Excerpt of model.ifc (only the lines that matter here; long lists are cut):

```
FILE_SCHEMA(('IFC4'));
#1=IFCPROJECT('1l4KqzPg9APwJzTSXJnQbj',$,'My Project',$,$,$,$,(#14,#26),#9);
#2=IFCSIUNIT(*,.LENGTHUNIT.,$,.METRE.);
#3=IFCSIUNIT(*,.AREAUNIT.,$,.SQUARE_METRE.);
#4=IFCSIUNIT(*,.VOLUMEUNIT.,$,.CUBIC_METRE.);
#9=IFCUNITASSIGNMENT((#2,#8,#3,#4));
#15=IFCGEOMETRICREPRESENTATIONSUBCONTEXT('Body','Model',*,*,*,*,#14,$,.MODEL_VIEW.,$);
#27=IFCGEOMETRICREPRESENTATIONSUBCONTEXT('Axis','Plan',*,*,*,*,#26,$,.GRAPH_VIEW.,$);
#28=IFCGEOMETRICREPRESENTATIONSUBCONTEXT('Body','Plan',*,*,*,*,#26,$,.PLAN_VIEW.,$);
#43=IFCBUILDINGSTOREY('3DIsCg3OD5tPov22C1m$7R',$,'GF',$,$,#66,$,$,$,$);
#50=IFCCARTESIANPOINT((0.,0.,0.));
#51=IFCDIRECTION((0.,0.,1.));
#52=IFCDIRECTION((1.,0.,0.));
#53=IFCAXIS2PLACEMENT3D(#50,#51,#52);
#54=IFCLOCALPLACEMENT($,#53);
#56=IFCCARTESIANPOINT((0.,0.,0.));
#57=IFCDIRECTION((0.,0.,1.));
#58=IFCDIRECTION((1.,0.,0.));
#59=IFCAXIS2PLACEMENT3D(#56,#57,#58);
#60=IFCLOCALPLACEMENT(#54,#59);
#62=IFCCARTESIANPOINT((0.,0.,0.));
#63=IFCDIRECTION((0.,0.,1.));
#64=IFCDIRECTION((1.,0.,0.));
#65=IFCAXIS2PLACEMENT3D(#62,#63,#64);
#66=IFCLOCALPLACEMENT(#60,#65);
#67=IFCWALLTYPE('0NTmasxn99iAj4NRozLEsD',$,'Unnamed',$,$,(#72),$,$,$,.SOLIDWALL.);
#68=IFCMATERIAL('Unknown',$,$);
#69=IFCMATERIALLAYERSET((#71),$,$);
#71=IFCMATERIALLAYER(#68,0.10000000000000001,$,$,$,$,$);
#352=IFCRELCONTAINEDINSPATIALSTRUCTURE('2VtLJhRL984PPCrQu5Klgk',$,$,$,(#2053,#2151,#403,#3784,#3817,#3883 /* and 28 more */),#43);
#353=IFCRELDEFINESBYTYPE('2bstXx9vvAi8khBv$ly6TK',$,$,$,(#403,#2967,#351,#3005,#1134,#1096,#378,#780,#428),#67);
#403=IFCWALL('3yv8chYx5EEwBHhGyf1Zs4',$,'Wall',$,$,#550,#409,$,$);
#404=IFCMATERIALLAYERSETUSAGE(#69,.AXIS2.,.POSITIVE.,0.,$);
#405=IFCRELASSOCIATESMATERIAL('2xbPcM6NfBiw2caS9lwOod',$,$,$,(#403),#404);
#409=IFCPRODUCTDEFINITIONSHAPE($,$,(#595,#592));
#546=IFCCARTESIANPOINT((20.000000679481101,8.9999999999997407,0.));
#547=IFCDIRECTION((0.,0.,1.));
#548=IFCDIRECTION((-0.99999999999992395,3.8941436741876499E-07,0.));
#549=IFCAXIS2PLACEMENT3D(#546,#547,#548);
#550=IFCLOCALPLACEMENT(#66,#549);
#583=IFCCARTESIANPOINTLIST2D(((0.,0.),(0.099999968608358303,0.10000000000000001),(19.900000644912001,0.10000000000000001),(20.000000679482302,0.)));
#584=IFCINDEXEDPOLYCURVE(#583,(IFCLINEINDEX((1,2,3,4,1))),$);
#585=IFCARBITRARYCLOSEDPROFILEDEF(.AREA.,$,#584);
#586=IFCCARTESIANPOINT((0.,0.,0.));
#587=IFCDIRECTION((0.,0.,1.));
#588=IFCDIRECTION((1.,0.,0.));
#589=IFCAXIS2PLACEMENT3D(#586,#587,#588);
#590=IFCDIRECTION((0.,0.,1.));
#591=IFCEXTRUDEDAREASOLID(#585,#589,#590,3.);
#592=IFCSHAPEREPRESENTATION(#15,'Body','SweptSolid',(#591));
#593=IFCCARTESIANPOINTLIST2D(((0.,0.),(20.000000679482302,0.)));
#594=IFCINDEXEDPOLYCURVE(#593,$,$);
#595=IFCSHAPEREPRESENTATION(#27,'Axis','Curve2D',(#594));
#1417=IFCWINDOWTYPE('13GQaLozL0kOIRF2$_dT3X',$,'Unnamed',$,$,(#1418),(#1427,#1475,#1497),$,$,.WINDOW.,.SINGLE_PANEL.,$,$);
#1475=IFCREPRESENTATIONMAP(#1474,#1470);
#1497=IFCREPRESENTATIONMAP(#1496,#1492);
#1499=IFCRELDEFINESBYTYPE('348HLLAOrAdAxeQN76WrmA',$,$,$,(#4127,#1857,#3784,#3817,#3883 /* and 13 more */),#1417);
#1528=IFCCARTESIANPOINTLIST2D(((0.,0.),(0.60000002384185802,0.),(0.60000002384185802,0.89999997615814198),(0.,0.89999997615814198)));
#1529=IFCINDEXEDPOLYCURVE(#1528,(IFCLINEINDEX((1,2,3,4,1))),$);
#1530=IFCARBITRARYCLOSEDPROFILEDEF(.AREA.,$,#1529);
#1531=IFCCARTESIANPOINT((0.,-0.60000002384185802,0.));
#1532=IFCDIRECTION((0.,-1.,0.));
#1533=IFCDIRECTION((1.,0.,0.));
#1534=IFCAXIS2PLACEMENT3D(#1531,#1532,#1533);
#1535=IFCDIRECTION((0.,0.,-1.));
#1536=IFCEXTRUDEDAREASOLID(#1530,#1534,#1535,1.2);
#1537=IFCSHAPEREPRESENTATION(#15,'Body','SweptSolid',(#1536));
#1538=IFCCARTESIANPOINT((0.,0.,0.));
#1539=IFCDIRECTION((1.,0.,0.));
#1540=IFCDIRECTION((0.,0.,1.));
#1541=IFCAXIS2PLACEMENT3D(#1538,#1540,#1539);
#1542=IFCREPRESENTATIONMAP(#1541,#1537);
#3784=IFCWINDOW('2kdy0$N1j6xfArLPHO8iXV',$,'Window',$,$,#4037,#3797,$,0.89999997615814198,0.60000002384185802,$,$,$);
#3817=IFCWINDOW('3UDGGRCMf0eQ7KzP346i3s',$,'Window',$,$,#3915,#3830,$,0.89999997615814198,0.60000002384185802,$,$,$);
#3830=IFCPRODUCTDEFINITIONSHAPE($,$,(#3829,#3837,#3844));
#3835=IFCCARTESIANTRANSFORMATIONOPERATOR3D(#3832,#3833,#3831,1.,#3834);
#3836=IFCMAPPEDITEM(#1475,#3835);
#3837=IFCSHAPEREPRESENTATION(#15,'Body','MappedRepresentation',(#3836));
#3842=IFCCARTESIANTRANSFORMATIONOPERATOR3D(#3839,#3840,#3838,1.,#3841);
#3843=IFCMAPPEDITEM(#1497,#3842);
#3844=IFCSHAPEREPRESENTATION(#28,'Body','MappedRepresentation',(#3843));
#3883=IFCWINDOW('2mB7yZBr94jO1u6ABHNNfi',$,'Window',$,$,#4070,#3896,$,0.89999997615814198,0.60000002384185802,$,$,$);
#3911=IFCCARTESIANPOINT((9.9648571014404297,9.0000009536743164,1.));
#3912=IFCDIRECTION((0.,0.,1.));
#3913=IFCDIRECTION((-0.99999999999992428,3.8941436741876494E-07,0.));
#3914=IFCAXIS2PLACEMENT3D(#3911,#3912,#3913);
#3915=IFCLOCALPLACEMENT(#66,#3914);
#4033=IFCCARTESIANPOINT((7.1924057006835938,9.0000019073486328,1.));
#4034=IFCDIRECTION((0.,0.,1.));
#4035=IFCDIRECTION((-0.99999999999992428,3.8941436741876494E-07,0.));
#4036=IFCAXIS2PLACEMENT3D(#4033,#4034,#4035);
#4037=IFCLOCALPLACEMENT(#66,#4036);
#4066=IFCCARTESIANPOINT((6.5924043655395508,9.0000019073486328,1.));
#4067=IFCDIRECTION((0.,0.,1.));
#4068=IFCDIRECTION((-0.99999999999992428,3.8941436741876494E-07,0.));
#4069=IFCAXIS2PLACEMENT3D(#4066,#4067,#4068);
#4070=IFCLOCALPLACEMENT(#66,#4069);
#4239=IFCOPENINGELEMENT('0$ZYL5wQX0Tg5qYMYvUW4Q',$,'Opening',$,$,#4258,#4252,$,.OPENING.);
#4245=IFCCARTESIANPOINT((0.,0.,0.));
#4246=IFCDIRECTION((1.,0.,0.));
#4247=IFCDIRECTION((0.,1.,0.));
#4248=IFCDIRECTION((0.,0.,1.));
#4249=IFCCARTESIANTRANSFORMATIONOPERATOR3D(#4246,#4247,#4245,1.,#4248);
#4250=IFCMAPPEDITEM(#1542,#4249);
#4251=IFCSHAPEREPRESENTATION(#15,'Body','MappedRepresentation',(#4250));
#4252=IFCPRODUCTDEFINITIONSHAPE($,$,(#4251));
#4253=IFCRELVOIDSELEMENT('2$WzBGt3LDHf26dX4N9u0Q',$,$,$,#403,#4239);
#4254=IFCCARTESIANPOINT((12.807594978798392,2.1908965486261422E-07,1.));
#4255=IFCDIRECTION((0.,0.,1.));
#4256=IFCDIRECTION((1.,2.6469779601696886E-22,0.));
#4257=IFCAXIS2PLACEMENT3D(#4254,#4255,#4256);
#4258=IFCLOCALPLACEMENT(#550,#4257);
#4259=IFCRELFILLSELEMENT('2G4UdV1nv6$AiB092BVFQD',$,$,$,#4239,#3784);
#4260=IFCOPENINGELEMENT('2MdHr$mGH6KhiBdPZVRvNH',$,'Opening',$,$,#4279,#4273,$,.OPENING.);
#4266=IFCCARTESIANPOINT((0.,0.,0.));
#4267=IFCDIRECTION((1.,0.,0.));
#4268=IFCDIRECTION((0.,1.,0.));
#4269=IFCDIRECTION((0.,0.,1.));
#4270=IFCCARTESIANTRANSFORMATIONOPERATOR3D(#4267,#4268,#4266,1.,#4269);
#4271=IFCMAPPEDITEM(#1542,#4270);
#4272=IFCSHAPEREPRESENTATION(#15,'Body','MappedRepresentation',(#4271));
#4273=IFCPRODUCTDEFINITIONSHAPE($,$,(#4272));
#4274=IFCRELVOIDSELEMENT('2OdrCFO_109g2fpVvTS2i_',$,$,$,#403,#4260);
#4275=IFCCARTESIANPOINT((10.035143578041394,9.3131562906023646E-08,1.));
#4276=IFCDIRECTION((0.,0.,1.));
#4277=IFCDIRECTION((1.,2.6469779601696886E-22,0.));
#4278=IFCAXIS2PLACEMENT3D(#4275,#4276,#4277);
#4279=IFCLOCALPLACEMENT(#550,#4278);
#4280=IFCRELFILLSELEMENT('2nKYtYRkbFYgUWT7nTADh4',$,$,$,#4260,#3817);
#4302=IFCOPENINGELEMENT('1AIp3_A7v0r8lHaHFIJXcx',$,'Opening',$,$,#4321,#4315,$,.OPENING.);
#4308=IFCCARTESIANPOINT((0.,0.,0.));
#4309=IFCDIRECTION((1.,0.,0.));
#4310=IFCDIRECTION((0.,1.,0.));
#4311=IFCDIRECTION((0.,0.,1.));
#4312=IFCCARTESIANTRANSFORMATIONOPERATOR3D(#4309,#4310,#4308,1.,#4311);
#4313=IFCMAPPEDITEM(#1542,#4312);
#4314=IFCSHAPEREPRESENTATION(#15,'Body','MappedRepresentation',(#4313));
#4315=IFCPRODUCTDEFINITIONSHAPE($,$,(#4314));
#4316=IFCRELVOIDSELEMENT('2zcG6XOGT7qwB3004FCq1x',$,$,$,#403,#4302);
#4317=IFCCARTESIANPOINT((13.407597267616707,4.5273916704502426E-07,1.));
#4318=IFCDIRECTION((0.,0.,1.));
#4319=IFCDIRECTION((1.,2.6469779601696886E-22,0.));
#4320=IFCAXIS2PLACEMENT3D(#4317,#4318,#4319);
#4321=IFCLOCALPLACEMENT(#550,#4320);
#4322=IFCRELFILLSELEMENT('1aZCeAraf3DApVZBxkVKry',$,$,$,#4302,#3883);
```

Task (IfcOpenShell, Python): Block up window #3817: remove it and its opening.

```python
import ifcopenshell
import ifcopenshell.api.feature
import ifcopenshell.api.root
import ifcopenshell.geom
import ifcopenshell.util.shape

model = ifcopenshell.open("model.ifc")
settings = ifcopenshell.geom.settings()


def volume(element):
    """Net volume in cubic metres, openings subtracted."""
    shape = ifcopenshell.geom.create_shape(settings, element)
    return ifcopenshell.util.shape.get_volume(shape.geometry)


window = model.by_id(3817)
opening = window.FillsVoids[0].RelatingOpeningElement
wall = opening.VoidsElements[0].RelatingBuildingElement
before = volume(wall)

ifcopenshell.api.root.remove_product(model, product=window)
ifcopenshell.api.feature.remove_feature(model, feature=opening)

after = volume(wall)

print(f"wall volume {before:.3f} -> {after:.3f} m3")

model.write("model_updated.ifc")
```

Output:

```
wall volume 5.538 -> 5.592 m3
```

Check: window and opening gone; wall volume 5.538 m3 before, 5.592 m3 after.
